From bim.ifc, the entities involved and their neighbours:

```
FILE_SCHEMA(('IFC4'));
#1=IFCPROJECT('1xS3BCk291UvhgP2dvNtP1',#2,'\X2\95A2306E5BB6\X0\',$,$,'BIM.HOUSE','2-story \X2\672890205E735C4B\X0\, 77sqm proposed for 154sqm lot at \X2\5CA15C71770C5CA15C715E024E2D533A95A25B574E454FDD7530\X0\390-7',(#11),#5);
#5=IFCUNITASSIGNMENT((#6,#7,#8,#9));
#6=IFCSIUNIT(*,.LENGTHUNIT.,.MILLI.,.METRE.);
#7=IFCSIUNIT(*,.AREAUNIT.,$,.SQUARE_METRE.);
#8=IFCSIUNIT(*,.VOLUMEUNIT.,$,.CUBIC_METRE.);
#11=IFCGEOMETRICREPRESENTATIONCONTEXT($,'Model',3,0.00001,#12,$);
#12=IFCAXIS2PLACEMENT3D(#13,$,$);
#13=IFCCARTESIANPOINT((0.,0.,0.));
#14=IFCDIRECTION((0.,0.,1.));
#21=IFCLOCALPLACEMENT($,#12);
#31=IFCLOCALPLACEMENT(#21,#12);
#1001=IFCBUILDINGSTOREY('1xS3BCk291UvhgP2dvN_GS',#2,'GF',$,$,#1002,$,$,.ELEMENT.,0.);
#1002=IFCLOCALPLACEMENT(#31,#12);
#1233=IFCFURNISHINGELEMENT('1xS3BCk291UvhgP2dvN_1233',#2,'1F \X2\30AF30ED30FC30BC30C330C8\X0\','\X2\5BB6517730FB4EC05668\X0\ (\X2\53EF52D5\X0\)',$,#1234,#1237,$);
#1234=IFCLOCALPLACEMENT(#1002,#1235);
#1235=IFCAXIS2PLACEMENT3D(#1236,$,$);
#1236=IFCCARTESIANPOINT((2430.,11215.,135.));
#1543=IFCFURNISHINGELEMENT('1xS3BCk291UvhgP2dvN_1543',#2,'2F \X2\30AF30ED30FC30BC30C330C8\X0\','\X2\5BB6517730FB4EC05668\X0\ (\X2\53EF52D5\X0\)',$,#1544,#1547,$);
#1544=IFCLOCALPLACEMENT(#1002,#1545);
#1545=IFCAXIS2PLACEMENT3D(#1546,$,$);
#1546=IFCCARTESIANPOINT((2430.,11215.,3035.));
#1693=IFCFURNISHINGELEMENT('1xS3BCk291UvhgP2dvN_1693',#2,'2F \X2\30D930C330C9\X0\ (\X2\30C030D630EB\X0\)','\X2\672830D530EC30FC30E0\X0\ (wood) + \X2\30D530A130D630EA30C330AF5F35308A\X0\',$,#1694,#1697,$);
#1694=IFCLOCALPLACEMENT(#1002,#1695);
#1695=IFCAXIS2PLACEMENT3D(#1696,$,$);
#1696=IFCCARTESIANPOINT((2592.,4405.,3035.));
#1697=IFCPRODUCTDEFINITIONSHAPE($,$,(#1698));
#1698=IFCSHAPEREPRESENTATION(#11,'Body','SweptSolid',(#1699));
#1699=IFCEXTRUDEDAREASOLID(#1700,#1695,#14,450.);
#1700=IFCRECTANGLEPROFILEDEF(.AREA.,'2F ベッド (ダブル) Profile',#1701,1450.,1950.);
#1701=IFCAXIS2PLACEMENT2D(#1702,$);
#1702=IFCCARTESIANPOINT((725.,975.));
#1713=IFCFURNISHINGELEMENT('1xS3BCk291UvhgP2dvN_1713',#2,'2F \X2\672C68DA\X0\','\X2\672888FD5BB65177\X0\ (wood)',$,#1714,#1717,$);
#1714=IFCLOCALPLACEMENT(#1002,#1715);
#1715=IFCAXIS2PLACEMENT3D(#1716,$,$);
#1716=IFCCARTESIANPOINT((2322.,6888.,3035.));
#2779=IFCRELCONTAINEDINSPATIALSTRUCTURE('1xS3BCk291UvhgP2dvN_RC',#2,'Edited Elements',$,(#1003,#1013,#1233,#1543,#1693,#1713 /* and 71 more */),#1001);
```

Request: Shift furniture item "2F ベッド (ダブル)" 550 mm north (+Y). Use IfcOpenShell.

```python
import ifcopenshell
import ifcopenshell.api.geometry
import ifcopenshell.util.placement
import ifcopenshell.util.unit

model = ifcopenshell.open("bim.ifc")
unit_scale = ifcopenshell.util.unit.calculate_unit_scale(model)

item = model.by_id(1693)
matrix = ifcopenshell.util.placement.get_local_placement(item.ObjectPlacement)
matrix[1, 3] += 0.55 / unit_scale
ifcopenshell.api.geometry.edit_object_placement(model, product=item, matrix=matrix, is_si=False)

print(ifcopenshell.util.placement.get_local_placement(item.ObjectPlacement).round(3) + 0.0)

model.write("bim_updated.ifc")
```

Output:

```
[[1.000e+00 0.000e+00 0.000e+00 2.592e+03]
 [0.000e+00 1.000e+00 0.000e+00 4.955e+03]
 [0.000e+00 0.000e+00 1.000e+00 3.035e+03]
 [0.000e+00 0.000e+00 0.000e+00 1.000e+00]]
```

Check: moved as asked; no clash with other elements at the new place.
